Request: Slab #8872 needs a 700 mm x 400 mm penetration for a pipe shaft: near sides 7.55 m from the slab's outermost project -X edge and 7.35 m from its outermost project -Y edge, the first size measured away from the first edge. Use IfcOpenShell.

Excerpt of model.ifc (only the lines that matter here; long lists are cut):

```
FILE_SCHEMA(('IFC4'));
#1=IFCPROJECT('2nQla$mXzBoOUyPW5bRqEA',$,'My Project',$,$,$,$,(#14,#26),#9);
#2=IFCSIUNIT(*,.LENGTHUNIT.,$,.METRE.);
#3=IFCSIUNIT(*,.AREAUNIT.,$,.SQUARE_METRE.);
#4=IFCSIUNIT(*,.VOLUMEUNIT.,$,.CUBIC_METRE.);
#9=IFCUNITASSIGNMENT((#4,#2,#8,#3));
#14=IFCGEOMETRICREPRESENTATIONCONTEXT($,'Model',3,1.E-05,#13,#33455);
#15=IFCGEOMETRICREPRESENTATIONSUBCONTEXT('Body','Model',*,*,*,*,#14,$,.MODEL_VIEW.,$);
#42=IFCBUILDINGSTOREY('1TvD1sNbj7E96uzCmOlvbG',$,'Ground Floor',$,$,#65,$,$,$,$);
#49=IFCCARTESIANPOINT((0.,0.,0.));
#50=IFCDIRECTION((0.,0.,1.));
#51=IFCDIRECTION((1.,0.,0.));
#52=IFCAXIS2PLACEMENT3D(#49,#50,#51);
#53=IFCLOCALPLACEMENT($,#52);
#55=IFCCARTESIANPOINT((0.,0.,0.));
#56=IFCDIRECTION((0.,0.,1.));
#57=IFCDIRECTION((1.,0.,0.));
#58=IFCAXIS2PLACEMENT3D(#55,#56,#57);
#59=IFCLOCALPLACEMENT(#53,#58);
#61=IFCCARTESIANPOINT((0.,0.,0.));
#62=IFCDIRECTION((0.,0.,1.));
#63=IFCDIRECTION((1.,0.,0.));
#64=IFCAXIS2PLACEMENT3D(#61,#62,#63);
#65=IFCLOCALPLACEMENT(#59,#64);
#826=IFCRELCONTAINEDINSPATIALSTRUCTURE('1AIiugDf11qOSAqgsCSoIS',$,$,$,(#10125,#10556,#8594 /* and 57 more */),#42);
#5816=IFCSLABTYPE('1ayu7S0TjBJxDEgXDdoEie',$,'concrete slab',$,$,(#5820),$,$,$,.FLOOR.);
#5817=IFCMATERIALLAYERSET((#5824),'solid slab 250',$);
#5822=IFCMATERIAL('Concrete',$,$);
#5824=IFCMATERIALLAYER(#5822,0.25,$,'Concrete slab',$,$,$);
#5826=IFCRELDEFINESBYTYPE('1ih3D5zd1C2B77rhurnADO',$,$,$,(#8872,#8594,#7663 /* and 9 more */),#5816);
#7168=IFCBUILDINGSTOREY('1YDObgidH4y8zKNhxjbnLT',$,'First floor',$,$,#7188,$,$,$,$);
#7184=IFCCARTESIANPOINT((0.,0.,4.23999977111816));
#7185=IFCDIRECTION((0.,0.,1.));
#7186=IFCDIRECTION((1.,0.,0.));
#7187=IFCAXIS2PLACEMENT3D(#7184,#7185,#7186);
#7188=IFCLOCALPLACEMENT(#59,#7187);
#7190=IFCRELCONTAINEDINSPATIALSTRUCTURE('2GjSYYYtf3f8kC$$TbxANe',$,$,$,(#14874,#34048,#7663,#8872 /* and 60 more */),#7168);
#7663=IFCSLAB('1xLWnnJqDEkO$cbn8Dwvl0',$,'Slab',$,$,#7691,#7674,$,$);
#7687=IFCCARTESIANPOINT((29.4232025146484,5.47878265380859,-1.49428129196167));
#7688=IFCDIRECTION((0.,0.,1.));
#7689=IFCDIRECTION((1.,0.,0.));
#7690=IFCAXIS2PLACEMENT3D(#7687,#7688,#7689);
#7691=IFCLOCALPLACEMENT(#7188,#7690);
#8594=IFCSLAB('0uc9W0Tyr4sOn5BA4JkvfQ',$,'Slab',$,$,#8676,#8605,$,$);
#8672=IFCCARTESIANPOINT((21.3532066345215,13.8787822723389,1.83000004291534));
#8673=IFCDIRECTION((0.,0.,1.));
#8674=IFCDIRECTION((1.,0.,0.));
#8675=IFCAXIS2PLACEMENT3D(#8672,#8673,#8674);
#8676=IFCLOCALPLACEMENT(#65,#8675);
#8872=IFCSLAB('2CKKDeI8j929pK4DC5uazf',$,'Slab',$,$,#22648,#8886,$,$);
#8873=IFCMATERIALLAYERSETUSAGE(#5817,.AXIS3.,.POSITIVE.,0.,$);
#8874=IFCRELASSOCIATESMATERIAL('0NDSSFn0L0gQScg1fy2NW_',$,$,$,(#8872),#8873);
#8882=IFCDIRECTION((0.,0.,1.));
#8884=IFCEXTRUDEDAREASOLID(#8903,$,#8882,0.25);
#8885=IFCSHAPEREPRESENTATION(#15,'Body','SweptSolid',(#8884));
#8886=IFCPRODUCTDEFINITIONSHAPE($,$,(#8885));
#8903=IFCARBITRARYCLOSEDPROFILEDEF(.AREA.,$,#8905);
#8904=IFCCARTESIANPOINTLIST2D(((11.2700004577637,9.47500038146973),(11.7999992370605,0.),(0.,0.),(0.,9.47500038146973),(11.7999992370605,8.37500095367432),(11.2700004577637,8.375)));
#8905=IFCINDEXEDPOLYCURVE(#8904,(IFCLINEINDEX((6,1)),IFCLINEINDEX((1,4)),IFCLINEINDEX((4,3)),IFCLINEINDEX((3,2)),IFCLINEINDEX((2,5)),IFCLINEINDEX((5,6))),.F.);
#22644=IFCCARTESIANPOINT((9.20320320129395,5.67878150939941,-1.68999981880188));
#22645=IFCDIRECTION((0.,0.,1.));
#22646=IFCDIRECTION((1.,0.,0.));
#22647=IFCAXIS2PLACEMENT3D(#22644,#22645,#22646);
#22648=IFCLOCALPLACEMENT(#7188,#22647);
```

```python
import numpy as np
import ifcopenshell
import ifcopenshell.api.feature
import ifcopenshell.api.geometry
import ifcopenshell.api.root
import ifcopenshell.geom
import ifcopenshell.util.placement
import ifcopenshell.util.representation
import ifcopenshell.util.shape
import ifcopenshell.util.unit

model = ifcopenshell.open("model.ifc")
unit_scale = ifcopenshell.util.unit.calculate_unit_scale(model)
settings = ifcopenshell.geom.settings()


def volume(element):
    """Net volume in cubic metres, openings subtracted."""
    shape = ifcopenshell.geom.create_shape(settings, element)
    return ifcopenshell.util.shape.get_volume(shape.geometry)


slab = model.by_id(8872)
before = volume(slab)

# Extent in the slab's own axes, in metres. The edges named are its -X and -Y sides.
slab_shape = ifcopenshell.geom.create_shape(settings, slab)
vertices = ifcopenshell.util.shape.get_vertices(slab_shape.geometry)
x_min, y_min, bottom = vertices.min(axis=0)
top = vertices[:, 2].max()

opening = ifcopenshell.api.root.create_entity(model, ifc_class="IfcOpeningElement", name="Pipe shaft opening", predefined_type="OPENING")
context = ifcopenshell.util.representation.get_context(model, "Model", "Body", "MODEL_VIEW")
width, depth = 0.7, 0.4
outline = [(0.0, 0.0), (width, 0.0), (width, depth), (0.0, depth), (0.0, 0.0)]
# Overshoot both faces by 50 mm so the cut is clean.
shape = ifcopenshell.api.geometry.add_slab_representation(
    model, context=context, depth=top - bottom + 0.1, polyline=outline
)
ifcopenshell.api.geometry.assign_representation(model, product=opening, representation=shape)

matrix = ifcopenshell.util.placement.get_local_placement(slab.ObjectPlacement)
matrix[:, 3] = matrix @ np.append(np.array([x_min + 7.55, y_min + 7.35, bottom - 0.05]) / unit_scale, 1.0)
ifcopenshell.api.geometry.edit_object_placement(model, product=opening, matrix=matrix, is_si=False)
ifcopenshell.api.feature.add_feature(model, feature=opening, element=slab)

after = volume(slab)

print(f"slab volume {before:.3f} -> {after:.3f} m3")

model.write("model_v2.ifc")
```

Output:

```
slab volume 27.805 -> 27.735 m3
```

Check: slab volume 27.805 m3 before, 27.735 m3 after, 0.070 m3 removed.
